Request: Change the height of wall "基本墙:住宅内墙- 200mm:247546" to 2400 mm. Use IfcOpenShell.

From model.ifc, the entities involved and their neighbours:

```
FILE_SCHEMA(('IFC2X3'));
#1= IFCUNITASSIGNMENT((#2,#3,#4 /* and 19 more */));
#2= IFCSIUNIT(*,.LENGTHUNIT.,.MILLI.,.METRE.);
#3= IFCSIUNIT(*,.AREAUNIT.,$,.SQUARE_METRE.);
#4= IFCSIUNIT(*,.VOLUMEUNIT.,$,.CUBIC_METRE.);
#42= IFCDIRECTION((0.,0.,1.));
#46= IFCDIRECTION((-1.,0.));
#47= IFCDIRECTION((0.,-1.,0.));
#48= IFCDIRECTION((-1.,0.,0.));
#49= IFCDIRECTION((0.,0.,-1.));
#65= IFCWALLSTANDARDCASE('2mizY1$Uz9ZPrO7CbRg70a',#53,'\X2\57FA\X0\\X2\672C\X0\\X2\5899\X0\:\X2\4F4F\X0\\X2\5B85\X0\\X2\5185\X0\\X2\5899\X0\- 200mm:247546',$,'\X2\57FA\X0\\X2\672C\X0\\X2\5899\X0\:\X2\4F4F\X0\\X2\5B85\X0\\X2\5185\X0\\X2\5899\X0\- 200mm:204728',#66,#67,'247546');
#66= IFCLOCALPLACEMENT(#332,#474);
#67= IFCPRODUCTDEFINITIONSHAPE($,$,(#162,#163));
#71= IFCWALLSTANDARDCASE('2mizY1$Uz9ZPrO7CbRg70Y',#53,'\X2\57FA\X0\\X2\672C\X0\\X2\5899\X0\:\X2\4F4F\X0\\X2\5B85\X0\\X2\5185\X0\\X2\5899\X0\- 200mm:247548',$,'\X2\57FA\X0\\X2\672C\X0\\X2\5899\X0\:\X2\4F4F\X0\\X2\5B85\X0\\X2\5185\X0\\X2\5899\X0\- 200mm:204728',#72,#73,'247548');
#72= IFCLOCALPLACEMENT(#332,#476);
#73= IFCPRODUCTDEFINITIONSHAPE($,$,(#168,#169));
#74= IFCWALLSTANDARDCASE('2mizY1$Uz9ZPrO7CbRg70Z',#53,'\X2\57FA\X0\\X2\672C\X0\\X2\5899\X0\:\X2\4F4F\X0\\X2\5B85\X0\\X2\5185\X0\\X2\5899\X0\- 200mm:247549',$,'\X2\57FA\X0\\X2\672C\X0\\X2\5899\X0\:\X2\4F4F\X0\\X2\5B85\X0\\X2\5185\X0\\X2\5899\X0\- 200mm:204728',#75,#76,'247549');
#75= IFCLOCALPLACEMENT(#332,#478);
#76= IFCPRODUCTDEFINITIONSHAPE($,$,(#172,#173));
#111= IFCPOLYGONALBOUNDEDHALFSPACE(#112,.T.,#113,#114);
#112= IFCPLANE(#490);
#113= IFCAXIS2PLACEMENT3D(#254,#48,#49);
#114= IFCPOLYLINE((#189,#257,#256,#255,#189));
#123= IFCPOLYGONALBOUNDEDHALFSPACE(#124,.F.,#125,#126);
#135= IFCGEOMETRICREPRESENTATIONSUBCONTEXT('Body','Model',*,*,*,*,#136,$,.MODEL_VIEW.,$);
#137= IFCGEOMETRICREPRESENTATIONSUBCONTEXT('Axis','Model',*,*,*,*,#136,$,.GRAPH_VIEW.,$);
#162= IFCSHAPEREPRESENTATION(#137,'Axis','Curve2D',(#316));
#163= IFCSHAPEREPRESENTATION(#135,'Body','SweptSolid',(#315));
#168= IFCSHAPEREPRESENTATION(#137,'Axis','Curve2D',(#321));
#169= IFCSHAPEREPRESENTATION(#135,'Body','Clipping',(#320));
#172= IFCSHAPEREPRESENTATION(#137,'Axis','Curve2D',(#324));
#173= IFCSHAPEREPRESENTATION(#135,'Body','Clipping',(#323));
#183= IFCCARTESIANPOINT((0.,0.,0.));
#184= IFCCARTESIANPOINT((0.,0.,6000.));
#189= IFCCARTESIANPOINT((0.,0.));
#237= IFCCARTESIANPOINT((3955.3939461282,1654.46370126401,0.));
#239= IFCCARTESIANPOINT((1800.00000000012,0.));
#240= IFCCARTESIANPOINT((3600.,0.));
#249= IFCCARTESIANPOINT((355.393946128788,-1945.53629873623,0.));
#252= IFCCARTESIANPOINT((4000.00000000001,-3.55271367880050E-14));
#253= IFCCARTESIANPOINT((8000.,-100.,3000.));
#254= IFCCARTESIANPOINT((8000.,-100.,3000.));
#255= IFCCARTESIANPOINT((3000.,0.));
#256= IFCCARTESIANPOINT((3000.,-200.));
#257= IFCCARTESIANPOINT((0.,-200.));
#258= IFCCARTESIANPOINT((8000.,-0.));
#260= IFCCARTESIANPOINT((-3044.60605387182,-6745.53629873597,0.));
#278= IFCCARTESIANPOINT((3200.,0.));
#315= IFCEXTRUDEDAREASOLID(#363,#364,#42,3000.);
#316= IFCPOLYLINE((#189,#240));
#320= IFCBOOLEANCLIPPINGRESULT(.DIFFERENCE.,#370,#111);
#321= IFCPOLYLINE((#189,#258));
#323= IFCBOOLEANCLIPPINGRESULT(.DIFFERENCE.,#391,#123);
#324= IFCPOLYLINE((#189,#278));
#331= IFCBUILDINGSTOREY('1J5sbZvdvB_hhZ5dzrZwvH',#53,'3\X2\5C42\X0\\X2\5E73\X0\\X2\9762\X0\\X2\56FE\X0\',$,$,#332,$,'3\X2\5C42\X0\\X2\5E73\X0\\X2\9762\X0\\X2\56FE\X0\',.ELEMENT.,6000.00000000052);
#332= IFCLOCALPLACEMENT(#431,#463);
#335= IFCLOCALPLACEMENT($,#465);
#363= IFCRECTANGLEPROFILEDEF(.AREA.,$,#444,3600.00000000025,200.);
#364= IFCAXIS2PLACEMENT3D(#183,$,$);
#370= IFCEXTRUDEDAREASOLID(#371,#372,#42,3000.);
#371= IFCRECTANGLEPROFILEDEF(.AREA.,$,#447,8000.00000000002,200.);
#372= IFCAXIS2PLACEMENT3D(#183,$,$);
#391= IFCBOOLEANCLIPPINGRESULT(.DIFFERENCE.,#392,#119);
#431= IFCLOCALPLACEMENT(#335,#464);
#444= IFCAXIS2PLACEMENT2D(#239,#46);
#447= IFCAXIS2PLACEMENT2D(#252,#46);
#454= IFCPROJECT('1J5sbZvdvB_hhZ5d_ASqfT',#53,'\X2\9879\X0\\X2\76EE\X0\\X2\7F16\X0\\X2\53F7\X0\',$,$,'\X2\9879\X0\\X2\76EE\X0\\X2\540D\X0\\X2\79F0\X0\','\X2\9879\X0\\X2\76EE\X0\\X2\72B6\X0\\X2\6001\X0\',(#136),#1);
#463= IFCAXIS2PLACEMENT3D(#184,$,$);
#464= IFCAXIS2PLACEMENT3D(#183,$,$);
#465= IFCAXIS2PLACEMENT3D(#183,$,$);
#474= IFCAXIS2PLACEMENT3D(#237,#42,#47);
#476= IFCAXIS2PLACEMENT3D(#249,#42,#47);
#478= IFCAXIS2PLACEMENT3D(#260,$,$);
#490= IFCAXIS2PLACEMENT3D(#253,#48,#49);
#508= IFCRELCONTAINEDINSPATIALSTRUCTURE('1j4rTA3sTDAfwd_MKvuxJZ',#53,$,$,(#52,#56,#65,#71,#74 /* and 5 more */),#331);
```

```python
import ifcopenshell
import ifcopenshell.geom
import ifcopenshell.util.representation
import ifcopenshell.util.shape
import ifcopenshell.util.unit

model = ifcopenshell.open("model.ifc")
unit_scale = ifcopenshell.util.unit.calculate_unit_scale(model)
settings = ifcopenshell.geom.settings()


def volume(element):
    """Net volume in cubic metres, openings subtracted."""
    shape = ifcopenshell.geom.create_shape(settings, element)
    return ifcopenshell.util.shape.get_volume(shape.geometry)


wall = model.by_guid("2mizY1$Uz9ZPrO7CbRg70a")
before = volume(wall)

body = ifcopenshell.util.representation.get_representation(wall, "Model", "Body")
solid = body.Items[0]
old_height = solid.Depth
solid.Depth = 2.4 / unit_scale
after = volume(wall)

print(f"height {old_height:g} -> {solid.Depth:g}, volume {before:.3f} -> {after:.3f} m3")

model.write("model-out.ifc")
```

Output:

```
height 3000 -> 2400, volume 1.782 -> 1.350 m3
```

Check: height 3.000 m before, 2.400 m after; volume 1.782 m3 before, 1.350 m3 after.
